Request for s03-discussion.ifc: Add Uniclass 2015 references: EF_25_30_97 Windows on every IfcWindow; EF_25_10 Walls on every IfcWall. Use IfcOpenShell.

First a look at what the model holds.

```python
import ifcopenshell

model = ifcopenshell.open("s03-discussion.ifc")
print(model.schema)
print("classifications:", [c.Name for c in model.by_type("IfcClassification")])
for ifc_class in ("IfcDoor", "IfcRoof", "IfcStair", "IfcWall", "IfcWindow"):
    print(ifc_class, len(model.by_type(ifc_class)))
```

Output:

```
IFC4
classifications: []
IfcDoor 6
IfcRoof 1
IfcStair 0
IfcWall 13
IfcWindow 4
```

```python
import ifcopenshell
import ifcopenshell.api.classification

model = ifcopenshell.open("s03-discussion.ifc")

system = ifcopenshell.api.classification.add_classification(model, classification="Uniclass 2015")

codes = {
    "IfcWindow": ("EF_25_30_97", "Windows"),
    "IfcWall": ("EF_25_10", "Walls"),
}
for ifc_class, (code, name) in codes.items():
    products = model.by_type(ifc_class)
    ifcopenshell.api.classification.add_reference(
        model, products=products, classification=system, identification=code, name=name
    )
    print(code, len(products))

model.write("s03-discussion-out.ifc")
```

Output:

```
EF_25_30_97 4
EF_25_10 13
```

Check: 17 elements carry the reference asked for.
